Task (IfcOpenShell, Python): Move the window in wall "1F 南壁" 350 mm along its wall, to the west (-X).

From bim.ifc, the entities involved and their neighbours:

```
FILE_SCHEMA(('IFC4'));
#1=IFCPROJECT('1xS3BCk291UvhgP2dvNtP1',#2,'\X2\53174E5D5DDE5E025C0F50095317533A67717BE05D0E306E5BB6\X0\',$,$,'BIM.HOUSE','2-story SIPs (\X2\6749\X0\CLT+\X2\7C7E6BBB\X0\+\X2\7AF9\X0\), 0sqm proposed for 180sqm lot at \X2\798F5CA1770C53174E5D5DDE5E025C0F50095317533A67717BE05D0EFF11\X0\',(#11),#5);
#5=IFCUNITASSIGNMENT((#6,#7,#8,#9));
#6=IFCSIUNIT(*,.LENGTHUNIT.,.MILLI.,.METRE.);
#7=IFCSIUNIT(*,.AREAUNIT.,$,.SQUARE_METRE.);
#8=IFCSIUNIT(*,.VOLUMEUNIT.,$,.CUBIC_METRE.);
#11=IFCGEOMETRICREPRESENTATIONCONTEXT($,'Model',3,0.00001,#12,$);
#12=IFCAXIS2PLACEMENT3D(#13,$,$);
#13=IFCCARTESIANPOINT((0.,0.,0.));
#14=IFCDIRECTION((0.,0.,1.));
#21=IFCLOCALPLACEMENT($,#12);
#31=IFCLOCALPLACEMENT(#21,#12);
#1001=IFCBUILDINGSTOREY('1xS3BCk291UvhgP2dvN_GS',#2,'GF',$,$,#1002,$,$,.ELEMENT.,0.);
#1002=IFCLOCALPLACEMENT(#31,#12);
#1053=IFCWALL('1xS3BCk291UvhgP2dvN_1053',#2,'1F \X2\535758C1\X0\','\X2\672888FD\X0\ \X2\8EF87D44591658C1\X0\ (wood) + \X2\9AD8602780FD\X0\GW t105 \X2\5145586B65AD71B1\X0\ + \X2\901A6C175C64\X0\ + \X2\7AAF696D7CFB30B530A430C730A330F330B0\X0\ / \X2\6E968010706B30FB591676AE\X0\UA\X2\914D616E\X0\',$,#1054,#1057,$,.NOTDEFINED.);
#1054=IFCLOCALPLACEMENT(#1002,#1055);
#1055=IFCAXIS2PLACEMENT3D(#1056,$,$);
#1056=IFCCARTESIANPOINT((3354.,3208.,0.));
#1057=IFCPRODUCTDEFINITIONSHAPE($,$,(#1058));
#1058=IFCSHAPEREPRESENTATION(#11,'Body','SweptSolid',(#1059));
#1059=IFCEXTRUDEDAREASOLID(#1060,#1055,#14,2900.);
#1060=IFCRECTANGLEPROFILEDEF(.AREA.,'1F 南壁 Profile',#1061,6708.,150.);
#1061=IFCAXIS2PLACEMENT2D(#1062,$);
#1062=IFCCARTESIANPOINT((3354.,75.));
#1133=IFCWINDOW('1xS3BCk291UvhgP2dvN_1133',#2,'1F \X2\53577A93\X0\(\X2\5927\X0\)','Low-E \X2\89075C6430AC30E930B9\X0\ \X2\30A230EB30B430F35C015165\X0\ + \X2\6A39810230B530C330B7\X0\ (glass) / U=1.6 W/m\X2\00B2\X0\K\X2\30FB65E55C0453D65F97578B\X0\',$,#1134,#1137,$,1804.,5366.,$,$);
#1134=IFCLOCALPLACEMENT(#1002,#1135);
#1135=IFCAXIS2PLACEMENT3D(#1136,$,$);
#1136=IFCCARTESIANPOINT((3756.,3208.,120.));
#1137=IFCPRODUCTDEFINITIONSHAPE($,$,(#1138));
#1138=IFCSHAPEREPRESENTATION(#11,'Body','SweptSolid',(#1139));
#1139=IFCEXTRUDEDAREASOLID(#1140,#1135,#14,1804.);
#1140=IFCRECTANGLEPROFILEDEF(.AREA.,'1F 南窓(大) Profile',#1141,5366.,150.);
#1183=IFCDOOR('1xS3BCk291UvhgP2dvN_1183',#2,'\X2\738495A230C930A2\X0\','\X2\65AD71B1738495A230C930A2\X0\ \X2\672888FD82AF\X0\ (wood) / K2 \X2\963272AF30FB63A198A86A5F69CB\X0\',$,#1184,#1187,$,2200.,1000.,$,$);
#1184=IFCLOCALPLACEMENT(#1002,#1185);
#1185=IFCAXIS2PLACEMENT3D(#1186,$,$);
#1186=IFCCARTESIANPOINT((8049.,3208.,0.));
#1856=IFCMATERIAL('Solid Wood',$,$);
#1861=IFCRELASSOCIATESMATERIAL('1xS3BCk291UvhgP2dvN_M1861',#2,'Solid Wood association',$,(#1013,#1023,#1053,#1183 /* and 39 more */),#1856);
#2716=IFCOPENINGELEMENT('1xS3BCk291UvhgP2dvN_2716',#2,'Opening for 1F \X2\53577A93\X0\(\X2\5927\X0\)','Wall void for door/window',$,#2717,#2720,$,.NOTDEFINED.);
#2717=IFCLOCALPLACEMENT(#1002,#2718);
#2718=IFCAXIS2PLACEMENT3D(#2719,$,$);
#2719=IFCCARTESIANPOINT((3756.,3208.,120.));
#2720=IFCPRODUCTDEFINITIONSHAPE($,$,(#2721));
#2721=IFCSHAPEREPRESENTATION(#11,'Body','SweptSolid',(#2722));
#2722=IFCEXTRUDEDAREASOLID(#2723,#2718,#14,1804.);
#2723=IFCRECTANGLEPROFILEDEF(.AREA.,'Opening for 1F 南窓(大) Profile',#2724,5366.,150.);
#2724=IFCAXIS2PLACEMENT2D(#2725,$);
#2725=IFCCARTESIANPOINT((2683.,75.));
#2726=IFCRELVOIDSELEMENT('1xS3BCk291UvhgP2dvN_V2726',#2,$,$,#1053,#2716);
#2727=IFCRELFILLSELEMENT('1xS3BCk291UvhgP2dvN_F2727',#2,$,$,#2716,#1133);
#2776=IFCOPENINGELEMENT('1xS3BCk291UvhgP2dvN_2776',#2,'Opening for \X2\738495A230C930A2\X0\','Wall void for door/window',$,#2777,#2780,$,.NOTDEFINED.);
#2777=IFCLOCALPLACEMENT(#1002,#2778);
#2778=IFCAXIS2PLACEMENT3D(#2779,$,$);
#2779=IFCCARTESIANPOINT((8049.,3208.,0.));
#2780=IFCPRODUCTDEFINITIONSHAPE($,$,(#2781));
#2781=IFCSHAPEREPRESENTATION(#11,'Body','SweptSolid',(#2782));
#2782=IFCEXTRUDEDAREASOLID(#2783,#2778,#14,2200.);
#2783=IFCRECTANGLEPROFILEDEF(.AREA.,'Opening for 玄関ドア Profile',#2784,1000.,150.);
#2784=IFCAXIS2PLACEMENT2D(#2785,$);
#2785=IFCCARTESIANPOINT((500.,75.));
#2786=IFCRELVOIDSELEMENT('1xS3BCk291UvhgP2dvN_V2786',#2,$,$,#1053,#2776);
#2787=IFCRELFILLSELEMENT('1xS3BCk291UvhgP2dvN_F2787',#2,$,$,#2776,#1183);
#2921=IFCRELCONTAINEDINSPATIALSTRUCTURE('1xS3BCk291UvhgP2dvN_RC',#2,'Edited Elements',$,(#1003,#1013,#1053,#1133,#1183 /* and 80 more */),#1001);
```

```python
import ifcopenshell
import ifcopenshell.api.geometry
import ifcopenshell.util.placement
import ifcopenshell.util.unit

model = ifcopenshell.open("bim.ifc")
unit_scale = ifcopenshell.util.unit.calculate_unit_scale(model)

window = model.by_guid("1xS3BCk291UvhgP2dvN_1133")
opening = window.FillsVoids[0].RelatingOpeningElement
wall = opening.VoidsElements[0].RelatingBuildingElement

wall_matrix = ifcopenshell.util.placement.get_local_placement(wall.ObjectPlacement)
shift = wall_matrix[:3, 0] * -0.35 / unit_scale
before = ifcopenshell.util.placement.get_local_placement(window.ObjectPlacement)[:3, 3].copy()

# The window is not placed relative to its opening, so move both.
for product in (opening, window):
    matrix = ifcopenshell.util.placement.get_local_placement(product.ObjectPlacement)
    matrix[:3, 3] += shift
    ifcopenshell.api.geometry.edit_object_placement(model, product=product, matrix=matrix, is_si=False)

after = ifcopenshell.util.placement.get_local_placement(window.ObjectPlacement)[:3, 3]
print("window moved by", (after - before).round(3) + 0.0)

model.write("bim-out.ifc")
```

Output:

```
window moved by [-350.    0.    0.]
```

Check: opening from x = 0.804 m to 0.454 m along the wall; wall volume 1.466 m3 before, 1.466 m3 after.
